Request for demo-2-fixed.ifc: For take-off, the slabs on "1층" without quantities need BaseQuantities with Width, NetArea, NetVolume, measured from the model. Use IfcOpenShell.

First a look at what the model holds.

```python
import ifcopenshell
import ifcopenshell.util.element
import ifcopenshell.util.unit

model = ifcopenshell.open("demo-2-fixed.ifc")
print(model.schema)
for unit_type in ("LENGTHUNIT", "AREAUNIT", "VOLUMEUNIT"):
    print(unit_type, ifcopenshell.util.unit.calculate_unit_scale(model, unit_type))
storey = next(s for s in model.by_type("IfcBuildingStorey") if s.Name == "1층")
slabs = [e for e in ifcopenshell.util.element.get_decomposition(storey) if e.is_a("IfcSlab")]
for e in sorted(slabs, key=lambda e: e.id()):
    print(e.id(), e.is_a(), e.Name, list(ifcopenshell.util.element.get_psets(e, qtos_only=True)), sep=" | ")
```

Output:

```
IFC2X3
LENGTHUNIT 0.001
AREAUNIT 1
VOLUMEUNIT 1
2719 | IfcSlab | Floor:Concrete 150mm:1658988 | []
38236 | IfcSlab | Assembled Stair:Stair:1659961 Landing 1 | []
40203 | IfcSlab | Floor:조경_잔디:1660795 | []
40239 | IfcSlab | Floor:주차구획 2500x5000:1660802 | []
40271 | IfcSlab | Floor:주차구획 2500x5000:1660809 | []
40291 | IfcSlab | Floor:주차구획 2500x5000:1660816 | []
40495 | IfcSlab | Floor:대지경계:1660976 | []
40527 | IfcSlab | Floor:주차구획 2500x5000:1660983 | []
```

```python
import ifcopenshell
import ifcopenshell.api.pset
import ifcopenshell.geom
import ifcopenshell.util.element
import ifcopenshell.util.shape
import ifcopenshell.util.unit

model = ifcopenshell.open("demo-2-fixed.ifc")
unit_scale = ifcopenshell.util.unit.calculate_unit_scale(model)
area_scale = ifcopenshell.util.unit.calculate_unit_scale(model, "AREAUNIT")
volume_scale = ifcopenshell.util.unit.calculate_unit_scale(model, "VOLUMEUNIT")
settings = ifcopenshell.geom.settings()

storey = next(s for s in model.by_type("IfcBuildingStorey") if s.Name == "1층")
slabs = [e for e in ifcopenshell.util.element.get_decomposition(storey) if e.is_a("IfcSlab")]

for e in sorted(slabs, key=lambda e: e.id()):
    if ifcopenshell.util.element.get_psets(e, qtos_only=True, should_inherit=False):
        continue
    # Geometry comes back in metres, in the element's own axes.
    shape = ifcopenshell.geom.create_shape(settings, e)
    values = {
        "Width": ifcopenshell.util.shape.get_z(shape.geometry) / unit_scale,
        "NetArea": ifcopenshell.util.shape.get_footprint_area(shape.geometry) / area_scale,
        "NetVolume": ifcopenshell.util.shape.get_volume(shape.geometry) / volume_scale,
    }
    qto = ifcopenshell.api.pset.add_qto(model, product=e, name="BaseQuantities")
    ifcopenshell.api.pset.edit_qto(model, qto=qto, properties=values)
    print(e.id(), {k: round(v, 3) for k, v in values.items()})

model.write("demo-2-fixed_edited.ifc")
```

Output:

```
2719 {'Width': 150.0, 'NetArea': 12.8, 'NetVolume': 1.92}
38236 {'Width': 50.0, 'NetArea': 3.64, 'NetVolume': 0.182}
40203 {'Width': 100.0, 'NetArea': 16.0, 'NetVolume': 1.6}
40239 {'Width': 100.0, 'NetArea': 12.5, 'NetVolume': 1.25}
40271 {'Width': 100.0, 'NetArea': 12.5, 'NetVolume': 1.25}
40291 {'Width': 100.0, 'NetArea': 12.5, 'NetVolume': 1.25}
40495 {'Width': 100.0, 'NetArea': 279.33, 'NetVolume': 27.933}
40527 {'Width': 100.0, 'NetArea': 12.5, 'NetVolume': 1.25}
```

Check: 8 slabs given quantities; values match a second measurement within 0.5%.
